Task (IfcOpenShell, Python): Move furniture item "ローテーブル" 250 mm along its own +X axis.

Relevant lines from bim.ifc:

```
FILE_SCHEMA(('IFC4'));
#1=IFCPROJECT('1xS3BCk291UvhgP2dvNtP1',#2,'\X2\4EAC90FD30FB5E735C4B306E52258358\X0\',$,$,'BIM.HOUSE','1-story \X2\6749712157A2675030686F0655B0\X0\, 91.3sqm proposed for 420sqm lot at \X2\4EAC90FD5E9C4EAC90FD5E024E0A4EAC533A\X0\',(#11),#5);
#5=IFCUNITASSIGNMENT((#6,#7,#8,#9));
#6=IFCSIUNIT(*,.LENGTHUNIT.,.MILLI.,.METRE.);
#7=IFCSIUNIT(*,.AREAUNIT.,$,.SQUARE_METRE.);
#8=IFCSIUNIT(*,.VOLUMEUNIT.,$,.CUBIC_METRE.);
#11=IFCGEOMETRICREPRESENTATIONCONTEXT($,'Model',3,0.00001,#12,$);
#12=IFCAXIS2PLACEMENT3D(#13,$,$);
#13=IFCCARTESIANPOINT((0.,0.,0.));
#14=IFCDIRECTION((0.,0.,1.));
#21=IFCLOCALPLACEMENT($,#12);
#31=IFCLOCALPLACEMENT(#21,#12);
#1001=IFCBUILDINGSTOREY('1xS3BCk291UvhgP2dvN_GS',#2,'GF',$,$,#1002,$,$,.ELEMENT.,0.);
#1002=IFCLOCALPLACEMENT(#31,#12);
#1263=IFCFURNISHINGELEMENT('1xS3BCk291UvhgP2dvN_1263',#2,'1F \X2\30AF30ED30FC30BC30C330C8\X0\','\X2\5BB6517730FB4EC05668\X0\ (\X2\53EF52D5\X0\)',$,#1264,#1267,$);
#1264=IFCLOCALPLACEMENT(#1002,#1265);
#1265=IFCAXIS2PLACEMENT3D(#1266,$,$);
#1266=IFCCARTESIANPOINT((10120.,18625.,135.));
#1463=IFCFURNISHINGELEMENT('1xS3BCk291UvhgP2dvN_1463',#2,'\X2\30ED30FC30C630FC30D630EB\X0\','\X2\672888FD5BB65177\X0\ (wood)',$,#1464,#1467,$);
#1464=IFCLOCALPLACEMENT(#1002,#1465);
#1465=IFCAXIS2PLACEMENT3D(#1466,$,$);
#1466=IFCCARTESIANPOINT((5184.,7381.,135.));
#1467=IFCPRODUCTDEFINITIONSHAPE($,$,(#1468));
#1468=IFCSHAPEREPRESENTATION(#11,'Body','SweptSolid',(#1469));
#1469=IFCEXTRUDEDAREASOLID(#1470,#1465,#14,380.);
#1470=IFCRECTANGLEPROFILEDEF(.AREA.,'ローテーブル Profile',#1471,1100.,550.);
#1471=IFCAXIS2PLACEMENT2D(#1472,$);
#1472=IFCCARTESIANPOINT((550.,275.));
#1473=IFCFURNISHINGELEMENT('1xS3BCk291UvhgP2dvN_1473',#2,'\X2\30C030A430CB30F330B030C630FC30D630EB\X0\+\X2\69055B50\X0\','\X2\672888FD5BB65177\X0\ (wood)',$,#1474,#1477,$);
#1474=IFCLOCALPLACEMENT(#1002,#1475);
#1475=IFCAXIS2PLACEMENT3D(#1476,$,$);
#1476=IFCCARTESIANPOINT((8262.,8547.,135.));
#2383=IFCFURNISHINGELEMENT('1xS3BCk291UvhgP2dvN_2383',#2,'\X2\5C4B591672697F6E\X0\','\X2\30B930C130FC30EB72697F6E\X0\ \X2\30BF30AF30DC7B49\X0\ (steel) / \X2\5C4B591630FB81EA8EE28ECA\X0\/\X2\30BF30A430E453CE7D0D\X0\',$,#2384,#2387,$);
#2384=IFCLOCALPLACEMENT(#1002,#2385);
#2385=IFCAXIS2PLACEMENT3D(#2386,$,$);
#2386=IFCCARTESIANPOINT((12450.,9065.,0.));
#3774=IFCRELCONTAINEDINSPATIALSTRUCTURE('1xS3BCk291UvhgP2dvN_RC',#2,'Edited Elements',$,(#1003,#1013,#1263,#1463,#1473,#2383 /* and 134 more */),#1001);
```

```python
import ifcopenshell
import ifcopenshell.api.geometry
import ifcopenshell.util.placement

model = ifcopenshell.open("bim.ifc")

item = model.by_guid("1xS3BCk291UvhgP2dvN_1463")
matrix = ifcopenshell.util.placement.get_local_placement(item.ObjectPlacement)
matrix[:3, 3] += matrix[:3, 0] * 250.0
ifcopenshell.api.geometry.edit_object_placement(model, product=item, matrix=matrix, is_si=False)

print(ifcopenshell.util.placement.get_local_placement(item.ObjectPlacement).round(3) + 0.0)

model.write("bim_edited.ifc")
```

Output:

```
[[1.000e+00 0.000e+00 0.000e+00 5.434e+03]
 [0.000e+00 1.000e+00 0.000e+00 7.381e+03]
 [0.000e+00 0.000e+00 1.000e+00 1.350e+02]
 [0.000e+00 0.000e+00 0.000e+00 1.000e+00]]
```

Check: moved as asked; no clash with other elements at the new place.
